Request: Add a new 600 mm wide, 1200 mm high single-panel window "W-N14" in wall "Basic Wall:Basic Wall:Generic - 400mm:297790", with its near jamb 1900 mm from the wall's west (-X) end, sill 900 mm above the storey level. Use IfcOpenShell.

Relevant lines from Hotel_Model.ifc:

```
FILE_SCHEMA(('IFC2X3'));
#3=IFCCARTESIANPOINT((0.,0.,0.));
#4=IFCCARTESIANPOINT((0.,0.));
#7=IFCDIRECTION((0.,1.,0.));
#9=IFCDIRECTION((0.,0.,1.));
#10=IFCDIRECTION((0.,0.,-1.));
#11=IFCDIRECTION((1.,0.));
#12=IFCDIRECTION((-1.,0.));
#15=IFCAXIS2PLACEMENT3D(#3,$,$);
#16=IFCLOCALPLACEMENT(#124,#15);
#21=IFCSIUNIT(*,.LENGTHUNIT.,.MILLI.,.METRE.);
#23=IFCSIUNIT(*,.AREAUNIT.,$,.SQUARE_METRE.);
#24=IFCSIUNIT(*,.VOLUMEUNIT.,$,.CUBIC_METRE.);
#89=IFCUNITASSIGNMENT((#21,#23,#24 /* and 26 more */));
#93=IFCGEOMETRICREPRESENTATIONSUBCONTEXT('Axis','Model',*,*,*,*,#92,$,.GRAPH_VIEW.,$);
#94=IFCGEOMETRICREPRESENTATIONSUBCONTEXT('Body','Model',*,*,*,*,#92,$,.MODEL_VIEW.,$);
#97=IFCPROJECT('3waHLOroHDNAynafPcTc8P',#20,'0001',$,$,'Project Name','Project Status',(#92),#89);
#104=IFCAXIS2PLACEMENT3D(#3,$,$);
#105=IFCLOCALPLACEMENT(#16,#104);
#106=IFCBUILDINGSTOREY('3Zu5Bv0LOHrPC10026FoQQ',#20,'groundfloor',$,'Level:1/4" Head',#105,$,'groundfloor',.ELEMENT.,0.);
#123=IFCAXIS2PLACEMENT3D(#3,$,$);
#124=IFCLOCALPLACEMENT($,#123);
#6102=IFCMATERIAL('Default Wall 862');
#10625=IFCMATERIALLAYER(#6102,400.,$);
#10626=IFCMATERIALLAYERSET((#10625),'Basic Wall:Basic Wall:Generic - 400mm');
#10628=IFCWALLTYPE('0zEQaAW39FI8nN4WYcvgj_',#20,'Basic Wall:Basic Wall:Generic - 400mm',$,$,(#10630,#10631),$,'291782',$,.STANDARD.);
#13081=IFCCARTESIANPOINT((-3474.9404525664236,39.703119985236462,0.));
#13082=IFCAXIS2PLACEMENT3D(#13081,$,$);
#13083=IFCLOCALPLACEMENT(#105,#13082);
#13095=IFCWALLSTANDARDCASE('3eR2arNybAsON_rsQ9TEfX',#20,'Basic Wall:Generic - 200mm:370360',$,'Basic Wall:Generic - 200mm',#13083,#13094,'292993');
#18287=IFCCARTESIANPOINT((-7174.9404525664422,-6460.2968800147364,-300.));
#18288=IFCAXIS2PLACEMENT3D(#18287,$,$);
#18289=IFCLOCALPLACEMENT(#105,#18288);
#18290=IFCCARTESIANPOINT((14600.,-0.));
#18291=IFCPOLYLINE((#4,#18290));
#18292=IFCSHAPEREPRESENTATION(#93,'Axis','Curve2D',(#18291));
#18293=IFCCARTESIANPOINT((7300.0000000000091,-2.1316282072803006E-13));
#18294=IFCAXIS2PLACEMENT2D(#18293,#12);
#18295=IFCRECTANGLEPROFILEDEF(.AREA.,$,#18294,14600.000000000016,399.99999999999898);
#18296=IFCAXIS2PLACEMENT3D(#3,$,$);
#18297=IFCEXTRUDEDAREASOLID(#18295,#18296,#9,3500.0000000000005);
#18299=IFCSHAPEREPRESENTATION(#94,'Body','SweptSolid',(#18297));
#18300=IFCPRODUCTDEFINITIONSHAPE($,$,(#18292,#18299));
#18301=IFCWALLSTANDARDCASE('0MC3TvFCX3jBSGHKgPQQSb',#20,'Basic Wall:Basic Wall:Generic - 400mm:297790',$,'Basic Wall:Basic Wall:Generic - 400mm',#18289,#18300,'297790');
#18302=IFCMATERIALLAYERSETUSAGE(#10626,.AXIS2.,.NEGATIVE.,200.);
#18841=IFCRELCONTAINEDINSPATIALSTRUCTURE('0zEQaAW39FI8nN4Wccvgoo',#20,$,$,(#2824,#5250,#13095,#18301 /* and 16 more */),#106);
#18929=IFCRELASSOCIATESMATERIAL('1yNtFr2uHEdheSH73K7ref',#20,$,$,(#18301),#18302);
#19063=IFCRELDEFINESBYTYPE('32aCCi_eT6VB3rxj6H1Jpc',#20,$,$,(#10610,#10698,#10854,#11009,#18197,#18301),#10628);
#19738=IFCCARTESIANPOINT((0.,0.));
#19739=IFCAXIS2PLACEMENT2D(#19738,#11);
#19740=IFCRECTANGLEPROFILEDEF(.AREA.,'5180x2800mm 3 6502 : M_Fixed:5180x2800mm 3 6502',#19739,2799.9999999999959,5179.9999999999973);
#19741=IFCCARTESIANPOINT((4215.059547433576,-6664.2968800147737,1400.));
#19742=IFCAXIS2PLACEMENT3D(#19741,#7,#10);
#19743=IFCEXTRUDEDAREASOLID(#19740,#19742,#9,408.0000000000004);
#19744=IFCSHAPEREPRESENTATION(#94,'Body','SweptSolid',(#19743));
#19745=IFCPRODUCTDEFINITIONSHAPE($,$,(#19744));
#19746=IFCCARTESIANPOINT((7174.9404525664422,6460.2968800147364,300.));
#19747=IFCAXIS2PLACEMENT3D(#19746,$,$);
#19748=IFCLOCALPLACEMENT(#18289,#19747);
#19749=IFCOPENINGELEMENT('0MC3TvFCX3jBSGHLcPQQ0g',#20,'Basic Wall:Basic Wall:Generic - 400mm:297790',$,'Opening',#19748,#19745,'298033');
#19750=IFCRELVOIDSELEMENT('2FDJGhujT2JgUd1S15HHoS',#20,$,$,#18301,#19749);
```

```python
import numpy as np
import ifcopenshell
import ifcopenshell.api.feature
import ifcopenshell.api.geometry
import ifcopenshell.api.root
import ifcopenshell.api.spatial
import ifcopenshell.api.type
import ifcopenshell.geom
import ifcopenshell.util.element
import ifcopenshell.util.placement
import ifcopenshell.util.representation
import ifcopenshell.util.shape
import ifcopenshell.util.unit

model = ifcopenshell.open("Hotel_Model.ifc")
unit_scale = ifcopenshell.util.unit.calculate_unit_scale(model)
settings = ifcopenshell.geom.settings()


def volume(element):
    """Net volume in cubic metres, openings subtracted."""
    shape = ifcopenshell.geom.create_shape(settings, element)
    return ifcopenshell.util.shape.get_volume(shape.geometry)


wall = model.by_id(18301)
storey = ifcopenshell.util.element.get_container(wall, ifc_class="IfcBuildingStorey")
context = ifcopenshell.util.representation.get_context(model, "Model", "Body", "MODEL_VIEW")
before = volume(wall)

width, height, from_end, sill = 0.6, 1.2, 1.9, 0.9  # metres

# The wall runs along its own X axis, and the end named is its -X end.
wall_shape = ifcopenshell.geom.create_shape(settings, wall)
x, y, z = ifcopenshell.util.shape.get_vertices(wall_shape.geometry).T
start = x.min() + from_end
face, thickness = float(y.min()), float(y.max() - y.min())
wall_matrix = ifcopenshell.util.placement.get_local_placement(wall.ObjectPlacement)
level = ifcopenshell.util.placement.get_local_placement(storey.ObjectPlacement)[2, 3]


def in_wall(x, y):
    """Placement at x, y metres in the wall's axes, at sill height."""
    matrix = wall_matrix.copy()
    matrix[:, 3] = wall_matrix @ np.array([x / unit_scale, y / unit_scale, 0.0, 1.0])
    matrix[2, 3] = level + sill / unit_scale
    return matrix


# Opening: a box that overshoots both wall faces by 50 mm.
opening = ifcopenshell.api.root.create_entity(model, ifc_class="IfcOpeningElement")
box = ifcopenshell.api.geometry.add_wall_representation(
    model, context=context, length=width, height=height, thickness=thickness + 0.1
)
ifcopenshell.api.geometry.assign_representation(model, product=opening, representation=box)
ifcopenshell.api.geometry.edit_object_placement(model, product=opening, matrix=in_wall(start, face - 0.05), is_si=False)
ifcopenshell.api.feature.add_feature(model, feature=opening, element=wall)

window = ifcopenshell.api.root.create_entity(model, ifc_class="IfcWindow", name="W-N14")
window.OverallWidth, window.OverallHeight = width / unit_scale, height / unit_scale
body = ifcopenshell.api.geometry.add_window_representation(
    model,
    context=context,
    overall_width=window.OverallWidth,
    overall_height=window.OverallHeight,
    partition_type="SINGLE_PANEL",
)
ifcopenshell.api.geometry.assign_representation(model, product=window, representation=body)
ifcopenshell.api.spatial.assign_container(model, products=[window], relating_structure=storey)
fills = ifcopenshell.api.feature.add_filling(model, opening=opening, element=window)
fills.OwnerHistory = window.OwnerHistory  # required in IFC2X3

# IFC2X3 keeps the operation on the window style.
style = ifcopenshell.api.root.create_entity(model, ifc_class="IfcWindowStyle", name="W-N14")
style.OperationType, style.ConstructionType = "SINGLE_PANEL", "NOTDEFINED"
style.ParameterTakesPrecedence = style.Sizeable = False
ifcopenshell.api.type.assign_type(model, related_objects=[window], relating_type=style)

# Centre the window in the wall's thickness.
ifcopenshell.api.geometry.edit_object_placement(model, product=window, matrix=in_wall(start, face), is_si=False)
window_shape = ifcopenshell.geom.create_shape(settings, window)
depth = ifcopenshell.util.shape.get_vertices(window_shape.geometry)[:, 1]
offset = face + thickness / 2 - (depth.min() + depth.max()) / 2
ifcopenshell.api.geometry.edit_object_placement(model, product=window, matrix=in_wall(start, offset), is_si=False)

after = volume(wall)

print(f"wall volume {before:.3f} -> {after:.3f} m3")

model.write("Hotel_Model_rev.ifc")
```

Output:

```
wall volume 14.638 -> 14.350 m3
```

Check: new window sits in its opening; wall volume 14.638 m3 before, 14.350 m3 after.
